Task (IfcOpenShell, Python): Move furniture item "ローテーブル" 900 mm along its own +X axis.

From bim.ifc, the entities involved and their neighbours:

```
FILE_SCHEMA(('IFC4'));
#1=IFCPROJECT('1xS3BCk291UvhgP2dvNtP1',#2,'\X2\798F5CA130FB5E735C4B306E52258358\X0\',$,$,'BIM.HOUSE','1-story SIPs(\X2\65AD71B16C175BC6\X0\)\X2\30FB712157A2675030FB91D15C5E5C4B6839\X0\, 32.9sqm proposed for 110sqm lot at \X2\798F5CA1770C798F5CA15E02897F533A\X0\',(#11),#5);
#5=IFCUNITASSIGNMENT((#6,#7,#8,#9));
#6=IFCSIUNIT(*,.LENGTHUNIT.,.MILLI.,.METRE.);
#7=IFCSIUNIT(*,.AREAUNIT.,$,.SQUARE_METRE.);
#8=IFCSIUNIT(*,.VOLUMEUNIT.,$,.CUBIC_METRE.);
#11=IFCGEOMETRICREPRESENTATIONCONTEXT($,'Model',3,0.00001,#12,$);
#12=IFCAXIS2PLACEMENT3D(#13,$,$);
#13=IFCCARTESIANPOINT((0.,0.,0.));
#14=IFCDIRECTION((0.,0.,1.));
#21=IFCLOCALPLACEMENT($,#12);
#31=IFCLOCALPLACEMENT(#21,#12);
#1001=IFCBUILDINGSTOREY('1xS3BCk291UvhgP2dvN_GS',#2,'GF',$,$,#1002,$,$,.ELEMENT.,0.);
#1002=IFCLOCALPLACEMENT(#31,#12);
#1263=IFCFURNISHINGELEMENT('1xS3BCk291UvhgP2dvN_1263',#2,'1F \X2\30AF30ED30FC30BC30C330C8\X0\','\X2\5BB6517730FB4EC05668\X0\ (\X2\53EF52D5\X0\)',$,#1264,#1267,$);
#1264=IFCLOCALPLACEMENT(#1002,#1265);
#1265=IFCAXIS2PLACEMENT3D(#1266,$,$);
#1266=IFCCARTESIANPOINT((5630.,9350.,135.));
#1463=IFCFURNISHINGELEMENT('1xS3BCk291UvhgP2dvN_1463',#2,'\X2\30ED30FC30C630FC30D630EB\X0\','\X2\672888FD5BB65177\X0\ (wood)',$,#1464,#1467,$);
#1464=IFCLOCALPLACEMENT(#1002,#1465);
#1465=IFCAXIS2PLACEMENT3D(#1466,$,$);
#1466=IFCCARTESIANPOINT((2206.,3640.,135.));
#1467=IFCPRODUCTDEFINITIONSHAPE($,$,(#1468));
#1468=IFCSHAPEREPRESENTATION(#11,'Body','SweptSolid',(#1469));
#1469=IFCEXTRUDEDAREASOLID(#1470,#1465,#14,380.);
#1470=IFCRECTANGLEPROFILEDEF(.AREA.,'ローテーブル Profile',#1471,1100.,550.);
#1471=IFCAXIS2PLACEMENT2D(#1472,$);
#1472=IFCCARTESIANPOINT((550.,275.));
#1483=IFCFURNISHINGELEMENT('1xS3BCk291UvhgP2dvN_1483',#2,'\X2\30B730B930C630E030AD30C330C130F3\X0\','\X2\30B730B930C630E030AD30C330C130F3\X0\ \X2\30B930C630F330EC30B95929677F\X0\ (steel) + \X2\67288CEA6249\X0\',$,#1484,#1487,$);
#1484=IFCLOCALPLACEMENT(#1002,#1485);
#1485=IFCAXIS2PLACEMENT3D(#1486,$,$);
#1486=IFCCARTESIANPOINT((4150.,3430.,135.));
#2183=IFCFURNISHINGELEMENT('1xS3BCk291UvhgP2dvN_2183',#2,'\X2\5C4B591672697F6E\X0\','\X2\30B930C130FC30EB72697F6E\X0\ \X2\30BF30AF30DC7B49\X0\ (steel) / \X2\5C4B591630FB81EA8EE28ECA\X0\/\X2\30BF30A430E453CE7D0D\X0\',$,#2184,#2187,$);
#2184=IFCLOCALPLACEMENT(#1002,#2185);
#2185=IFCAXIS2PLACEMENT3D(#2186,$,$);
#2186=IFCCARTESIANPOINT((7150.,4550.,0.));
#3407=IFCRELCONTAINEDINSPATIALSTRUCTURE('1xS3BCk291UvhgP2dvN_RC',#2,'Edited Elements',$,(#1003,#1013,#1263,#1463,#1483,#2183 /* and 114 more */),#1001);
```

```python
import ifcopenshell
import ifcopenshell.api.geometry
import ifcopenshell.util.placement
import ifcopenshell.util.unit

model = ifcopenshell.open("bim.ifc")
unit_scale = ifcopenshell.util.unit.calculate_unit_scale(model)

item = model.by_guid("1xS3BCk291UvhgP2dvN_1463")
matrix = ifcopenshell.util.placement.get_local_placement(item.ObjectPlacement)
matrix[:3, 3] += matrix[:3, 0] * 0.9 / unit_scale
ifcopenshell.api.geometry.edit_object_placement(model, product=item, matrix=matrix, is_si=False)

print(ifcopenshell.util.placement.get_local_placement(item.ObjectPlacement).round(3) + 0.0)

model.write("bim_edited.ifc")
```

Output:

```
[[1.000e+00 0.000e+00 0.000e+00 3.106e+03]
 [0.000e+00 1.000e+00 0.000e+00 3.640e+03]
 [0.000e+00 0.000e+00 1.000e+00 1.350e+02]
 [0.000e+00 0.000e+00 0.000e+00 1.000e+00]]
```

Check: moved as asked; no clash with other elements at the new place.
